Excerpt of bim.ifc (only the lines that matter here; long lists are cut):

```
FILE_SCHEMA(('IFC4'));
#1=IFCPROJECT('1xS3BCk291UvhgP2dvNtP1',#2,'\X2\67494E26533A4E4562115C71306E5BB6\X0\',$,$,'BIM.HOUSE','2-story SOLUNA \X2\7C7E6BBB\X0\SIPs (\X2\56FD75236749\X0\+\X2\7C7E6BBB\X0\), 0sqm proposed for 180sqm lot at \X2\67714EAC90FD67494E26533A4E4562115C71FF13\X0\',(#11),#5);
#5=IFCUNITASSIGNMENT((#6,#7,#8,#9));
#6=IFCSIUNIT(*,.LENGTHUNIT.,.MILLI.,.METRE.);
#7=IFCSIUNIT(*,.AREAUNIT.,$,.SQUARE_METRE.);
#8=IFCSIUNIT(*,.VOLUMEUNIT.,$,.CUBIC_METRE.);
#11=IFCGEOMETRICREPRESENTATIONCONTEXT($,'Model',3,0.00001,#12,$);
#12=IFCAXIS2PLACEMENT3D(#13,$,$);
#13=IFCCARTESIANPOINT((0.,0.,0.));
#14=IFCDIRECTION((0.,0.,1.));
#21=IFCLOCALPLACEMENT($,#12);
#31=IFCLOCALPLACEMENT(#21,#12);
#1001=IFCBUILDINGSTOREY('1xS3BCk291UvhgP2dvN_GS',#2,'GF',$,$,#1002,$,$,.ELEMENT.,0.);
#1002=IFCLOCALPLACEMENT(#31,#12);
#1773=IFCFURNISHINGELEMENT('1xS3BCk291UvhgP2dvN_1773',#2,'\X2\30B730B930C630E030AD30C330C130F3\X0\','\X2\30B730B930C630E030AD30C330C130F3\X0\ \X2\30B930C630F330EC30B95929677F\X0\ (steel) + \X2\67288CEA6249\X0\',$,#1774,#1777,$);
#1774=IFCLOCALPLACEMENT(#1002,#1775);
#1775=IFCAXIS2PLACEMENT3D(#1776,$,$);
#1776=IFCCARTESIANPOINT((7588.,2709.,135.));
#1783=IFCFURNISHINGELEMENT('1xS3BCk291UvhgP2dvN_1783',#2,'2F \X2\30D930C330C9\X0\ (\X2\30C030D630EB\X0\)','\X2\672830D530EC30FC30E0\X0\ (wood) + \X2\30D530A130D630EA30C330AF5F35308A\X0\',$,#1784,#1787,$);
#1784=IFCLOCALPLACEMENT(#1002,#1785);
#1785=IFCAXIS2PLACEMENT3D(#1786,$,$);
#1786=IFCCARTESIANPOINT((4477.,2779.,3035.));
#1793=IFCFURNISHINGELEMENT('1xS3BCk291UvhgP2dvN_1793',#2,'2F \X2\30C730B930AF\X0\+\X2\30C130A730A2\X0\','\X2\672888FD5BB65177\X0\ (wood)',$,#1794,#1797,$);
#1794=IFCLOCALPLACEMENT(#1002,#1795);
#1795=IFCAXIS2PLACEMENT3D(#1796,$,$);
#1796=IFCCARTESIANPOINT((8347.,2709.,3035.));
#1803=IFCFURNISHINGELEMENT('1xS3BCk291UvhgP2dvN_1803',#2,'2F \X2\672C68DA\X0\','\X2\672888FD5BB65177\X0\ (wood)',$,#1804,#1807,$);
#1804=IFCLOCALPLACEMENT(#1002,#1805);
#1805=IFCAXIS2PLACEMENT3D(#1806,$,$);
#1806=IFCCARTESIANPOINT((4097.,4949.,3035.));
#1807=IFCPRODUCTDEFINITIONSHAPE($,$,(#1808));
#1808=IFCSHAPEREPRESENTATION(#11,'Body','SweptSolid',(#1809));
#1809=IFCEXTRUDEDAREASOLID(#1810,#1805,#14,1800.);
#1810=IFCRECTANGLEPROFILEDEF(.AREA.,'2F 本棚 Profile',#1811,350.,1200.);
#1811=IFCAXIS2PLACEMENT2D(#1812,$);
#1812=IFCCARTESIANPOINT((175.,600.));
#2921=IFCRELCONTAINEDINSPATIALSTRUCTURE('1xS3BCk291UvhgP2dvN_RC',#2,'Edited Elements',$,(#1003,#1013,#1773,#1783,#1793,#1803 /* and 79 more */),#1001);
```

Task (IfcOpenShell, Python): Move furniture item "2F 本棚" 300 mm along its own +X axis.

```python
import ifcopenshell
import ifcopenshell.api.geometry
import ifcopenshell.util.placement
import ifcopenshell.util.unit

model = ifcopenshell.open("bim.ifc")
unit_scale = ifcopenshell.util.unit.calculate_unit_scale(model)

item = model.by_guid("1xS3BCk291UvhgP2dvN_1803")
matrix = ifcopenshell.util.placement.get_local_placement(item.ObjectPlacement)
matrix[:3, 3] += matrix[:3, 0] * 0.3 / unit_scale
ifcopenshell.api.geometry.edit_object_placement(model, product=item, matrix=matrix, is_si=False)

print(ifcopenshell.util.placement.get_local_placement(item.ObjectPlacement).round(3) + 0.0)

model.write("bim_rev.ifc")
```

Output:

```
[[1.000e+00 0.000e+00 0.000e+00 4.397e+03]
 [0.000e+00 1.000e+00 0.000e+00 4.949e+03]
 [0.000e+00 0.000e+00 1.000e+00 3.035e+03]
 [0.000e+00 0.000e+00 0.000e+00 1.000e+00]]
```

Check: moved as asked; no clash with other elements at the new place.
